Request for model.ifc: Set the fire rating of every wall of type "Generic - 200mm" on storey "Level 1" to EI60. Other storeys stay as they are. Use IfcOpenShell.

First a look at what the model holds.

```python
import ifcopenshell
import ifcopenshell.util.element

model = ifcopenshell.open("model.ifc")
print(model.schema)
storey = next(s for s in model.by_type("IfcBuildingStorey") if s.Name == "Level 1")
walls = [e for e in ifcopenshell.util.element.get_decomposition(storey) if e.is_a("IfcWall")]
seen = {}
for e in walls:
    element_type = ifcopenshell.util.element.get_type(e)
    key = (element_type.Name if element_type != e and element_type else None, ifcopenshell.util.element.get_pset(e, "Pset_WallCommon", "FireRating"))
    seen[key] = seen.get(key, 0) + 1
for (name, value), count in sorted(seen.items(), key=str):
    print(count, "x", name, "|", value)
```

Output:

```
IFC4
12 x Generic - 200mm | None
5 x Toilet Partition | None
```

```python
import ifcopenshell
import ifcopenshell.api.pset
import ifcopenshell.util.element

model = ifcopenshell.open("model.ifc")

storey = next(s for s in model.by_type("IfcBuildingStorey") if s.Name == "Level 1")
walls = [e for e in ifcopenshell.util.element.get_decomposition(storey) if e.is_a("IfcWall")]

count = 0
for e in walls:
    element_type = ifcopenshell.util.element.get_type(e)
    if element_type in (None, e) or element_type.Name != "Generic - 200mm":
        continue
    # add_pset returns the element's existing set when there is one.
    pset = ifcopenshell.api.pset.add_pset(model, product=e, name="Pset_WallCommon")
    ifcopenshell.api.pset.edit_pset(model, pset=pset, properties={"FireRating": "EI60"})
    count += 1

print(count, "walls updated")

model.write("model_v2.ifc")
```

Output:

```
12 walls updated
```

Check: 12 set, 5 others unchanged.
